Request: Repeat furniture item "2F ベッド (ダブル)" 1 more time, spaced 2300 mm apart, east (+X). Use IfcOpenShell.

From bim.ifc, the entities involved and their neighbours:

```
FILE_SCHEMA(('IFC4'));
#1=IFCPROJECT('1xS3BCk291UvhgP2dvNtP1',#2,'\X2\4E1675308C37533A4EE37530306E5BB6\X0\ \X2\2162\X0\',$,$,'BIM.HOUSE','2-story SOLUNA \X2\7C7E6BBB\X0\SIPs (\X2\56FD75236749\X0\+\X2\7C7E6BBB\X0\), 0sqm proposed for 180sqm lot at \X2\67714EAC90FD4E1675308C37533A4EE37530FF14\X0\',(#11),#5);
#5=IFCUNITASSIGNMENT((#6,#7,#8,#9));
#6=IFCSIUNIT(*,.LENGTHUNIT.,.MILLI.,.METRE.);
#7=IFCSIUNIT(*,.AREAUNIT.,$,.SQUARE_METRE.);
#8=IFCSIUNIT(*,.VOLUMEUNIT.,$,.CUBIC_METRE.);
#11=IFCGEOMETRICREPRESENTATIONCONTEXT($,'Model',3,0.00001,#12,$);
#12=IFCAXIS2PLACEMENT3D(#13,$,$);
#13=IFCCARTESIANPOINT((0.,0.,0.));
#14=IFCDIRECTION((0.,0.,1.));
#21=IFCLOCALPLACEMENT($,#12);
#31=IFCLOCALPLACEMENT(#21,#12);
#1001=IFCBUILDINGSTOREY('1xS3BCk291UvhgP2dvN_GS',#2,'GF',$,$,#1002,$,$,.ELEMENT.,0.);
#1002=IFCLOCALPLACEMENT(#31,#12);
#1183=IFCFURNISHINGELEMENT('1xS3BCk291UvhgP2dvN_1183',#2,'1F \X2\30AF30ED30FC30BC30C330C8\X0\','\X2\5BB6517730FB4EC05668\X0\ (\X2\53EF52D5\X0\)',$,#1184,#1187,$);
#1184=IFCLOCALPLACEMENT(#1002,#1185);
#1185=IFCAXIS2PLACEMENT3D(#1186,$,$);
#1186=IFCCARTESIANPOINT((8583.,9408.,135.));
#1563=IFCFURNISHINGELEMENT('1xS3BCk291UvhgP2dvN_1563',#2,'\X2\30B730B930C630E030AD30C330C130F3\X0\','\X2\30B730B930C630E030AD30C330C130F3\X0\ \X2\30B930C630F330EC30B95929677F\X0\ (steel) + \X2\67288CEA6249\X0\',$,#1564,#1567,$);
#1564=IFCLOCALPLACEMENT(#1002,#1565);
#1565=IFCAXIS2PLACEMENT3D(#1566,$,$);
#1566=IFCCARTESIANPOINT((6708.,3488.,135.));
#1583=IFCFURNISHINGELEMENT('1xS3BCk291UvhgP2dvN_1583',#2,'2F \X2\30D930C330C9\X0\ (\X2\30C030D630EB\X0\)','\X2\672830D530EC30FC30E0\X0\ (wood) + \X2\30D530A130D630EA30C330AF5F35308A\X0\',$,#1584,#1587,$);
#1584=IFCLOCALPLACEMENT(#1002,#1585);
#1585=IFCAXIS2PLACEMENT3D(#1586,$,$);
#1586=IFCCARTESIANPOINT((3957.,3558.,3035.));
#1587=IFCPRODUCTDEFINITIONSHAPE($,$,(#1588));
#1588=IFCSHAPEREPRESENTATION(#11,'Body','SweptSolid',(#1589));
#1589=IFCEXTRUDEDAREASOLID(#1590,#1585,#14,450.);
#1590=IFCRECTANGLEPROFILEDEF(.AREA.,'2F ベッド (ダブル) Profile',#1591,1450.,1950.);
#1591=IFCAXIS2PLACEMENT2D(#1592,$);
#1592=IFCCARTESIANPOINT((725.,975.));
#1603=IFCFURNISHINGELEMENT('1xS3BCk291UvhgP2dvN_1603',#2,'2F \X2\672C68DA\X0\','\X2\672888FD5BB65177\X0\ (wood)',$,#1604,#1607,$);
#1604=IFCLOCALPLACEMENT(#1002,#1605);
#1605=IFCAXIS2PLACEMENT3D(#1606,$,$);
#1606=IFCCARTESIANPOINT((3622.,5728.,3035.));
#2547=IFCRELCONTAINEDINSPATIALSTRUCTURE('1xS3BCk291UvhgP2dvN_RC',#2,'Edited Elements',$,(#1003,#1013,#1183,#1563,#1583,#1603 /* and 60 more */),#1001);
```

```python
import numpy as np
import ifcopenshell
import ifcopenshell.api.geometry
import ifcopenshell.api.root
import ifcopenshell.util.element
import ifcopenshell.util.placement
import ifcopenshell.util.unit

model = ifcopenshell.open("bim.ifc")
unit_scale = ifcopenshell.util.unit.calculate_unit_scale(model)


def reuse_history(source, copy):
    """copy_class also copies each property set's owner history, people and application; keep the originals."""
    for rel in copy.IsDefinedBy:
        if rel.is_a("IfcRelDefinesByProperties") and (history := rel.RelatingPropertyDefinition.OwnerHistory):
            rel.RelatingPropertyDefinition.OwnerHistory = source.OwnerHistory
            ifcopenshell.util.element.remove_deep2(model, history)


source = model.by_id(1583)
base = ifcopenshell.util.placement.get_local_placement(source.ObjectPlacement)
step = np.array([1.0, 0.0, 0.0]) * 2.3 / unit_scale

for i in range(1, 2):
    copy = ifcopenshell.api.root.copy_class(model, product=source)
    copy.Representation = ifcopenshell.util.element.copy_deep(
        model, source.Representation, exclude=["IfcGeometricRepresentationContext", "IfcRepresentationMap"]
    )
    reuse_history(source, copy)
    matrix = base.copy()
    matrix[:3, 3] += i * step
    print("added at", matrix[:3, 3].round(3) + 0.0)
    ifcopenshell.api.geometry.edit_object_placement(model, product=copy, matrix=matrix, is_si=False)

model.write("bim_updated.ifc")
```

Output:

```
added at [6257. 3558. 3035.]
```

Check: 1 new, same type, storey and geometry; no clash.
